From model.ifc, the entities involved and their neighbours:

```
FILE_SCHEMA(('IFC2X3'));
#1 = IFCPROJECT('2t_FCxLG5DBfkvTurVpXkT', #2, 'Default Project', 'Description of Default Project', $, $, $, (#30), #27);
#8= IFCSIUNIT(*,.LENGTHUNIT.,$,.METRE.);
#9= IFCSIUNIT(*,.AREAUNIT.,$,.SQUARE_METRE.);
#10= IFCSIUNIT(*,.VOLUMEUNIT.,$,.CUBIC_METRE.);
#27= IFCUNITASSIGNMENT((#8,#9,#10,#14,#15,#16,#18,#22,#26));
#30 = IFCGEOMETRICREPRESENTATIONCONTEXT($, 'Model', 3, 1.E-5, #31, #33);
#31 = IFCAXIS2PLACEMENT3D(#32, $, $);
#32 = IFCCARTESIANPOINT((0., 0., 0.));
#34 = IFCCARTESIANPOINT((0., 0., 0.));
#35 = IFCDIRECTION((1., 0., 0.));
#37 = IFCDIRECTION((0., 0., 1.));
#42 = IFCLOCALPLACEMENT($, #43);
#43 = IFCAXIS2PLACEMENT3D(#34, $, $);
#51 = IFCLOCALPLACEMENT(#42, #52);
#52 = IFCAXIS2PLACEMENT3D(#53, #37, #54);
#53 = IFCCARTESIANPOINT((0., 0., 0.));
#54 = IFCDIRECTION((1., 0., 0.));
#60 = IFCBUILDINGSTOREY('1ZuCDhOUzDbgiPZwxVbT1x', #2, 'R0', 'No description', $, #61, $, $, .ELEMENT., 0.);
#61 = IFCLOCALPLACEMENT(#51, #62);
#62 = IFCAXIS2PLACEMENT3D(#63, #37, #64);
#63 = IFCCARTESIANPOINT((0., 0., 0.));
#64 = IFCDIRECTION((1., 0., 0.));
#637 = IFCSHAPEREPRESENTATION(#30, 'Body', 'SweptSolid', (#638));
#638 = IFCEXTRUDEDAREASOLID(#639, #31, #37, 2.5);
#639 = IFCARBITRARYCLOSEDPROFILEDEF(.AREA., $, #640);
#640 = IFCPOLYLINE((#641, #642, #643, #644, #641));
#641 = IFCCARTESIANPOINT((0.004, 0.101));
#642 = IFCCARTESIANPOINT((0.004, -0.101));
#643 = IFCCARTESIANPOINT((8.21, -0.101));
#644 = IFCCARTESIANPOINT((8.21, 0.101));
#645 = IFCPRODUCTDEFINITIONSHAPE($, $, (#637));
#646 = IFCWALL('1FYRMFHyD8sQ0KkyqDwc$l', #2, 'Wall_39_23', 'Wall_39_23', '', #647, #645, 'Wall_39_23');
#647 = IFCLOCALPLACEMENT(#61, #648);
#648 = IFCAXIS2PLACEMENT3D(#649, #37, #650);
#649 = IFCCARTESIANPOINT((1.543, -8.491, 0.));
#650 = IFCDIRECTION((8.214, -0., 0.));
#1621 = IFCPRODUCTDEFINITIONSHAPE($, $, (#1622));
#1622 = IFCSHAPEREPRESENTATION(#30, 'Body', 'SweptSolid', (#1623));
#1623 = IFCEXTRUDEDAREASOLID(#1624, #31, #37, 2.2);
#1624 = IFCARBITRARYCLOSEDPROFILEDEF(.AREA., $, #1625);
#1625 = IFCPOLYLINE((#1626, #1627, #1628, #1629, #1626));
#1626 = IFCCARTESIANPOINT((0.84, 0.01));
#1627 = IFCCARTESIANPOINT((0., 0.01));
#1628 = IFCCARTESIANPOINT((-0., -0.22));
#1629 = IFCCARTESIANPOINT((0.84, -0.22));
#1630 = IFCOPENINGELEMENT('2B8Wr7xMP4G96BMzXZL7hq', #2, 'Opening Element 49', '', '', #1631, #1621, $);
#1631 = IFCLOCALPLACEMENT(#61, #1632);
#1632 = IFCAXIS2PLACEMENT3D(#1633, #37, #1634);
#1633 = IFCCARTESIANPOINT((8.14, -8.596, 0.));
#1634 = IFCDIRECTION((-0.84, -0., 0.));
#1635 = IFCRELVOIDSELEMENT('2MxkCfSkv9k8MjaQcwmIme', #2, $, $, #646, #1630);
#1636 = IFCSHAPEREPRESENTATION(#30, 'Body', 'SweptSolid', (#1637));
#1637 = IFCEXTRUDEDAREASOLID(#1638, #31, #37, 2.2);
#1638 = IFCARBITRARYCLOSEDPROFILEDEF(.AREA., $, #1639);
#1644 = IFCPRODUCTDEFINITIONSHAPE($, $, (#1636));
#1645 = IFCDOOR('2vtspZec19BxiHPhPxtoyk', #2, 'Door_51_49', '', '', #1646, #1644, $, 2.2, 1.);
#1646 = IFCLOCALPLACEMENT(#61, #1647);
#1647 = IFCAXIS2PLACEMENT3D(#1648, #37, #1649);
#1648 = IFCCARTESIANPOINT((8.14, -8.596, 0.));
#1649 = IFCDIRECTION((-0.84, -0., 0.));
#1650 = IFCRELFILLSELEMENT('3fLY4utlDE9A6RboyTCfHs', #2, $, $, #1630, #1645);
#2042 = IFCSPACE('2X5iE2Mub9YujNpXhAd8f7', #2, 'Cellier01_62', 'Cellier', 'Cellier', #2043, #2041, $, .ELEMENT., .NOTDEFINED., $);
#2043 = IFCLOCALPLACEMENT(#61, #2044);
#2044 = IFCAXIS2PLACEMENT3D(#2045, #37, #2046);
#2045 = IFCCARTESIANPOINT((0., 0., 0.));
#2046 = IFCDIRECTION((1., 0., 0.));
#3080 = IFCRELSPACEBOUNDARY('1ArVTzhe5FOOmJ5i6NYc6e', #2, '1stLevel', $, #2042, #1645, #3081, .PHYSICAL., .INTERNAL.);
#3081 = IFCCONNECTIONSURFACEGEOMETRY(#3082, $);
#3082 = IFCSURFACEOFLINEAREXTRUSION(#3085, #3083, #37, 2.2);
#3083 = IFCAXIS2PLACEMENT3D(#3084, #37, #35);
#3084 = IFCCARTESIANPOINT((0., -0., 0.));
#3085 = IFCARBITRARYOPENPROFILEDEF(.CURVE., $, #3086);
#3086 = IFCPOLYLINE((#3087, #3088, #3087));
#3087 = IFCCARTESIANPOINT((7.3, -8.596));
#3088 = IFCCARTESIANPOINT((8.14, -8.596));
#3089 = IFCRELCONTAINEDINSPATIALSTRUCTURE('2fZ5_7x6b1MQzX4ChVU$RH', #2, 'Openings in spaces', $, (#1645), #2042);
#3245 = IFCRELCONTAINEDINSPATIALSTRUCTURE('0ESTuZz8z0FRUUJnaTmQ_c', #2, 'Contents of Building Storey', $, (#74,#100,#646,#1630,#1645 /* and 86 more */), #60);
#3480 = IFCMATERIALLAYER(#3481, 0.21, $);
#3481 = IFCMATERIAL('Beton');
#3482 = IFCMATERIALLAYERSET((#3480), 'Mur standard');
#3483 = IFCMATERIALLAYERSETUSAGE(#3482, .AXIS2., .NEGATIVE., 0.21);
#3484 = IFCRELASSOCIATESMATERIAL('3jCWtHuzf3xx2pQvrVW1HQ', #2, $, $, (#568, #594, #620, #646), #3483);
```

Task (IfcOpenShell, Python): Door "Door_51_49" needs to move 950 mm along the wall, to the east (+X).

```python
import numpy as np
import ifcopenshell
import ifcopenshell.api.geometry
import ifcopenshell.util.placement
import ifcopenshell.util.unit

model = ifcopenshell.open("model.ifc")
unit_scale = ifcopenshell.util.unit.calculate_unit_scale(model)

door = model.by_id(1645)
opening = door.FillsVoids[0].RelatingOpeningElement
wall = opening.VoidsElements[0].RelatingBuildingElement

wall_matrix = ifcopenshell.util.placement.get_local_placement(wall.ObjectPlacement)
shift = wall_matrix[:3, 0] * 0.95 / unit_scale
before = ifcopenshell.util.placement.get_local_placement(door.ObjectPlacement)[:3, 3].copy()

# The door is not placed relative to its opening, so move both.
for product in (opening, door):
    matrix = ifcopenshell.util.placement.get_local_placement(product.ObjectPlacement)
    matrix[:3, 3] += shift
    ifcopenshell.api.geometry.edit_object_placement(model, product=product, matrix=matrix, is_si=False)

# Space boundary surfaces are stored in each space's coordinates; move them too.
for rel in door.ProvidesBoundaries:
    if not rel.ConnectionGeometry:
        continue
    surface = rel.ConnectionGeometry.SurfaceOnRelatingElement
    space_matrix = ifcopenshell.util.placement.get_local_placement(rel.RelatingSpace.ObjectPlacement)
    point = np.array(surface.Position.Location.Coordinates) + space_matrix[:3, :3].T @ shift
    surface.Position = model.createIfcAxis2Placement3D(
        model.createIfcCartesianPoint(point.tolist()), surface.Position.Axis, surface.Position.RefDirection
    )

after = ifcopenshell.util.placement.get_local_placement(door.ObjectPlacement)[:3, 3]
print("door moved by", (after - before).round(3) + 0.0)

model.write("model_v2.ifc")
```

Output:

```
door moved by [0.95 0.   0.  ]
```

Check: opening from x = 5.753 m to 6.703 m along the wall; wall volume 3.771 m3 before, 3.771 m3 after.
